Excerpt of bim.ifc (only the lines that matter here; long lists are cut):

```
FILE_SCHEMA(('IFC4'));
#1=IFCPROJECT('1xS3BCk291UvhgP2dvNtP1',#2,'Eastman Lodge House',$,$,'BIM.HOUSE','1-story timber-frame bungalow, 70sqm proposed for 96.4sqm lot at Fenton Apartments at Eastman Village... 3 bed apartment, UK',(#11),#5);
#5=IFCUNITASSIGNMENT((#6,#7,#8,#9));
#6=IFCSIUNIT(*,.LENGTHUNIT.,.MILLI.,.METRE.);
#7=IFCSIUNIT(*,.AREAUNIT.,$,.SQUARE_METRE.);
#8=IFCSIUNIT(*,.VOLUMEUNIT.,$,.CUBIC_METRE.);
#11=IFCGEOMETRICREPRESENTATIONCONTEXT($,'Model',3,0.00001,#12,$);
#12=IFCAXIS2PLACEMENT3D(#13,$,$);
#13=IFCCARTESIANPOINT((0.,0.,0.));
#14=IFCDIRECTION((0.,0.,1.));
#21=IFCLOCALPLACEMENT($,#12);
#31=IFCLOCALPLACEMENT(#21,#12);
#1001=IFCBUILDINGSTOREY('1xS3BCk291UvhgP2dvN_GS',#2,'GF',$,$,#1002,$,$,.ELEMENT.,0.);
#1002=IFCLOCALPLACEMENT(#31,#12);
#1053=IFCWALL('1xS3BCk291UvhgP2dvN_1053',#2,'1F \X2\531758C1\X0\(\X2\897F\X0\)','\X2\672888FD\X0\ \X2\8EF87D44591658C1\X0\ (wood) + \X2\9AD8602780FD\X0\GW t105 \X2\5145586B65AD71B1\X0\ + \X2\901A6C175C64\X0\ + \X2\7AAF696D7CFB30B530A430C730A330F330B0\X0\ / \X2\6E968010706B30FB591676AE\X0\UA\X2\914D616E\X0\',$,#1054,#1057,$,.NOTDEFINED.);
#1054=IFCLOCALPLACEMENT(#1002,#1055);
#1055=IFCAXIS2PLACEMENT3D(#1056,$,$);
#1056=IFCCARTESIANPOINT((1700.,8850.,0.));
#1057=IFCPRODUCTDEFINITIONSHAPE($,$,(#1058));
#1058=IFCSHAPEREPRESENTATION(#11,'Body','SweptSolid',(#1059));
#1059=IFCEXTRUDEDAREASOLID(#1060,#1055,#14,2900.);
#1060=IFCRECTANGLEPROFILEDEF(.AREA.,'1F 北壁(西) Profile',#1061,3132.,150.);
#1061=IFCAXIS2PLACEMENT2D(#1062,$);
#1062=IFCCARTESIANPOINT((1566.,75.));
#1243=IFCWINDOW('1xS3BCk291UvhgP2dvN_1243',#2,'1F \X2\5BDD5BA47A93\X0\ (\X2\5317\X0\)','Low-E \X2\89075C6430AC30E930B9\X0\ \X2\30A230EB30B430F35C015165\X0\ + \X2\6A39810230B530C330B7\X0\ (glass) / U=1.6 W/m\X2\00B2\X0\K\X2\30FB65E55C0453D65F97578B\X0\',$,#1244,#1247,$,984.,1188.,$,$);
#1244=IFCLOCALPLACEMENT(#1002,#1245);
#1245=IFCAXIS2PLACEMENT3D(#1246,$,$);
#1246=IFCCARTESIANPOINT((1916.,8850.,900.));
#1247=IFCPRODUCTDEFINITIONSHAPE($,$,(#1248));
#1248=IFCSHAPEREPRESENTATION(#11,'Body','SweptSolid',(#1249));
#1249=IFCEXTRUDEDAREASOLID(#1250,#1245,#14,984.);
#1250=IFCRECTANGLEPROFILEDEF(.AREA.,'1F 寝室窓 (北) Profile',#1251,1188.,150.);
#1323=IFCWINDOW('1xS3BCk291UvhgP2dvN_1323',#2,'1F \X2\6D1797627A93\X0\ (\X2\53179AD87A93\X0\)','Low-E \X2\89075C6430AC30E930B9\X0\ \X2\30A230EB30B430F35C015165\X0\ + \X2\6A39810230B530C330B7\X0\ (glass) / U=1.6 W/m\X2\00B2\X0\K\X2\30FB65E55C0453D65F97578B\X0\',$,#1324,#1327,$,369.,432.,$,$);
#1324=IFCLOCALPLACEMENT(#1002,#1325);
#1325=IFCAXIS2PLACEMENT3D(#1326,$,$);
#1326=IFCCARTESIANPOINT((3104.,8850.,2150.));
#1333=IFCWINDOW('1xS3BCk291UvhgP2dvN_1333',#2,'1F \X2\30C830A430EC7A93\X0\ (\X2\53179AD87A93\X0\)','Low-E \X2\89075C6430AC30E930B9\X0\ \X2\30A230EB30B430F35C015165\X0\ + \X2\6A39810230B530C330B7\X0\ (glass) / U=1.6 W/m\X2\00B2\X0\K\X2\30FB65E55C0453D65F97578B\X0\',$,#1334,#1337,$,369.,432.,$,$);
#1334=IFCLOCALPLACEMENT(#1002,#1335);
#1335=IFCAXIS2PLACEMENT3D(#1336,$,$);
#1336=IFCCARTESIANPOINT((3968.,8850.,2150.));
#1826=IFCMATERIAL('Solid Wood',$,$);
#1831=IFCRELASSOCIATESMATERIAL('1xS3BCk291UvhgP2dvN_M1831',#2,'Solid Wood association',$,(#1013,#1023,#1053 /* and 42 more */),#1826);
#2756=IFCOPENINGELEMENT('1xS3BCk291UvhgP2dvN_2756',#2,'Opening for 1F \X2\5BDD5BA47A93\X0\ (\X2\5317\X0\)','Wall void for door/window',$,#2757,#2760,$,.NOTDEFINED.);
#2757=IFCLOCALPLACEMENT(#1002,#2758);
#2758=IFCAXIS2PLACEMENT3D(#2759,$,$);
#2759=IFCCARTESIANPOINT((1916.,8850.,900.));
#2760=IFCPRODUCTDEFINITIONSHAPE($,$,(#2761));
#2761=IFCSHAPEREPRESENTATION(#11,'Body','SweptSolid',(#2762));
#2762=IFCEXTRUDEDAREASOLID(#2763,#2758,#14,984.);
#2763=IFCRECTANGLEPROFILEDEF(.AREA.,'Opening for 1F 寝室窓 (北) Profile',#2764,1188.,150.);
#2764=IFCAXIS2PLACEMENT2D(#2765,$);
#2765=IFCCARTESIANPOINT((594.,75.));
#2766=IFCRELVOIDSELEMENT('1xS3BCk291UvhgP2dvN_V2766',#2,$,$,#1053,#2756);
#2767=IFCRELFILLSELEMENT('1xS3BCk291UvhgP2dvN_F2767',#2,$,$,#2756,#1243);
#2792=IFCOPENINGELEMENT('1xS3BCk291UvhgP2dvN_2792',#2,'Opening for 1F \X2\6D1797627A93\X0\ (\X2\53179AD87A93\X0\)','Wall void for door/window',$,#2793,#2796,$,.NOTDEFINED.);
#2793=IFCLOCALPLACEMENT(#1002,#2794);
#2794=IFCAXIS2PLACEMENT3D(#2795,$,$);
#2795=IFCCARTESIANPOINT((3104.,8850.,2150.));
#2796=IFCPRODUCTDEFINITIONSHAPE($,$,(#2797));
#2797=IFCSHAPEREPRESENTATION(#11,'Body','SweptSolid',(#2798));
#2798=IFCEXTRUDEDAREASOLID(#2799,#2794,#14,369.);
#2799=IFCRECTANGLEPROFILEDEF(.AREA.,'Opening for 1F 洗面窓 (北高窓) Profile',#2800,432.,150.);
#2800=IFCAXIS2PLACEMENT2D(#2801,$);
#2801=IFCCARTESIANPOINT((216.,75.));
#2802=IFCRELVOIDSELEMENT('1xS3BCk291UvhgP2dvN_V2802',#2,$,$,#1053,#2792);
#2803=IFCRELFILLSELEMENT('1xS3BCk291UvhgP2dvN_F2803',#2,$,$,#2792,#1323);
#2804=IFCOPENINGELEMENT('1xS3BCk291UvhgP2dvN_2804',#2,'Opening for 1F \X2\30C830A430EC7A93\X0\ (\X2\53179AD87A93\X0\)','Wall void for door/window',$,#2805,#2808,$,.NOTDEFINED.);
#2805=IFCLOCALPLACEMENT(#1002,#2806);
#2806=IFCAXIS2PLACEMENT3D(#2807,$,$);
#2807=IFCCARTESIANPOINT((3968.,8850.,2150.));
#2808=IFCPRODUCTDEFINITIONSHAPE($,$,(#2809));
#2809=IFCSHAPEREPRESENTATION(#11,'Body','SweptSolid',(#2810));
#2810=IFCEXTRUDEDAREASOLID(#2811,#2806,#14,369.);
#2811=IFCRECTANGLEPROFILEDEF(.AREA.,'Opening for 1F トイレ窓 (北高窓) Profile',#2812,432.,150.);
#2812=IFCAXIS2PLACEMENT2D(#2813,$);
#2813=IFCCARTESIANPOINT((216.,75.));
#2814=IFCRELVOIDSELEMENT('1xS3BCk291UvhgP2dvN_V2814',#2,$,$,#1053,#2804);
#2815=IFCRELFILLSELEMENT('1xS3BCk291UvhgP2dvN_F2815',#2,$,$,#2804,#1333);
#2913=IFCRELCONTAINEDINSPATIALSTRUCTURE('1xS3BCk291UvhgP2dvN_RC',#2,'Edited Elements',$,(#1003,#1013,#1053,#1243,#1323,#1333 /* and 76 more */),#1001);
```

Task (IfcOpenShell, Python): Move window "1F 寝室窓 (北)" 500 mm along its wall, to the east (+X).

```python
import ifcopenshell
import ifcopenshell.api.geometry
import ifcopenshell.util.placement
import ifcopenshell.util.unit

model = ifcopenshell.open("bim.ifc")
unit_scale = ifcopenshell.util.unit.calculate_unit_scale(model)

window = model.by_id(1243)
opening = window.FillsVoids[0].RelatingOpeningElement
wall = opening.VoidsElements[0].RelatingBuildingElement

wall_matrix = ifcopenshell.util.placement.get_local_placement(wall.ObjectPlacement)
shift = wall_matrix[:3, 0] * 0.5 / unit_scale
before = ifcopenshell.util.placement.get_local_placement(window.ObjectPlacement)[:3, 3].copy()

# The window is not placed relative to its opening, so move both.
for product in (opening, window):
    matrix = ifcopenshell.util.placement.get_local_placement(product.ObjectPlacement)
    matrix[:3, 3] += shift
    ifcopenshell.api.geometry.edit_object_placement(model, product=product, matrix=matrix, is_si=False)

after = ifcopenshell.util.placement.get_local_placement(window.ObjectPlacement)[:3, 3]
print("window moved by", (after - before).round(3) + 0.0)

model.write("bim_updated.ifc")
```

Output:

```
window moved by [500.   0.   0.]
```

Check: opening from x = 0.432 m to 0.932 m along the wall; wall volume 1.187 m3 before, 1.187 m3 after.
